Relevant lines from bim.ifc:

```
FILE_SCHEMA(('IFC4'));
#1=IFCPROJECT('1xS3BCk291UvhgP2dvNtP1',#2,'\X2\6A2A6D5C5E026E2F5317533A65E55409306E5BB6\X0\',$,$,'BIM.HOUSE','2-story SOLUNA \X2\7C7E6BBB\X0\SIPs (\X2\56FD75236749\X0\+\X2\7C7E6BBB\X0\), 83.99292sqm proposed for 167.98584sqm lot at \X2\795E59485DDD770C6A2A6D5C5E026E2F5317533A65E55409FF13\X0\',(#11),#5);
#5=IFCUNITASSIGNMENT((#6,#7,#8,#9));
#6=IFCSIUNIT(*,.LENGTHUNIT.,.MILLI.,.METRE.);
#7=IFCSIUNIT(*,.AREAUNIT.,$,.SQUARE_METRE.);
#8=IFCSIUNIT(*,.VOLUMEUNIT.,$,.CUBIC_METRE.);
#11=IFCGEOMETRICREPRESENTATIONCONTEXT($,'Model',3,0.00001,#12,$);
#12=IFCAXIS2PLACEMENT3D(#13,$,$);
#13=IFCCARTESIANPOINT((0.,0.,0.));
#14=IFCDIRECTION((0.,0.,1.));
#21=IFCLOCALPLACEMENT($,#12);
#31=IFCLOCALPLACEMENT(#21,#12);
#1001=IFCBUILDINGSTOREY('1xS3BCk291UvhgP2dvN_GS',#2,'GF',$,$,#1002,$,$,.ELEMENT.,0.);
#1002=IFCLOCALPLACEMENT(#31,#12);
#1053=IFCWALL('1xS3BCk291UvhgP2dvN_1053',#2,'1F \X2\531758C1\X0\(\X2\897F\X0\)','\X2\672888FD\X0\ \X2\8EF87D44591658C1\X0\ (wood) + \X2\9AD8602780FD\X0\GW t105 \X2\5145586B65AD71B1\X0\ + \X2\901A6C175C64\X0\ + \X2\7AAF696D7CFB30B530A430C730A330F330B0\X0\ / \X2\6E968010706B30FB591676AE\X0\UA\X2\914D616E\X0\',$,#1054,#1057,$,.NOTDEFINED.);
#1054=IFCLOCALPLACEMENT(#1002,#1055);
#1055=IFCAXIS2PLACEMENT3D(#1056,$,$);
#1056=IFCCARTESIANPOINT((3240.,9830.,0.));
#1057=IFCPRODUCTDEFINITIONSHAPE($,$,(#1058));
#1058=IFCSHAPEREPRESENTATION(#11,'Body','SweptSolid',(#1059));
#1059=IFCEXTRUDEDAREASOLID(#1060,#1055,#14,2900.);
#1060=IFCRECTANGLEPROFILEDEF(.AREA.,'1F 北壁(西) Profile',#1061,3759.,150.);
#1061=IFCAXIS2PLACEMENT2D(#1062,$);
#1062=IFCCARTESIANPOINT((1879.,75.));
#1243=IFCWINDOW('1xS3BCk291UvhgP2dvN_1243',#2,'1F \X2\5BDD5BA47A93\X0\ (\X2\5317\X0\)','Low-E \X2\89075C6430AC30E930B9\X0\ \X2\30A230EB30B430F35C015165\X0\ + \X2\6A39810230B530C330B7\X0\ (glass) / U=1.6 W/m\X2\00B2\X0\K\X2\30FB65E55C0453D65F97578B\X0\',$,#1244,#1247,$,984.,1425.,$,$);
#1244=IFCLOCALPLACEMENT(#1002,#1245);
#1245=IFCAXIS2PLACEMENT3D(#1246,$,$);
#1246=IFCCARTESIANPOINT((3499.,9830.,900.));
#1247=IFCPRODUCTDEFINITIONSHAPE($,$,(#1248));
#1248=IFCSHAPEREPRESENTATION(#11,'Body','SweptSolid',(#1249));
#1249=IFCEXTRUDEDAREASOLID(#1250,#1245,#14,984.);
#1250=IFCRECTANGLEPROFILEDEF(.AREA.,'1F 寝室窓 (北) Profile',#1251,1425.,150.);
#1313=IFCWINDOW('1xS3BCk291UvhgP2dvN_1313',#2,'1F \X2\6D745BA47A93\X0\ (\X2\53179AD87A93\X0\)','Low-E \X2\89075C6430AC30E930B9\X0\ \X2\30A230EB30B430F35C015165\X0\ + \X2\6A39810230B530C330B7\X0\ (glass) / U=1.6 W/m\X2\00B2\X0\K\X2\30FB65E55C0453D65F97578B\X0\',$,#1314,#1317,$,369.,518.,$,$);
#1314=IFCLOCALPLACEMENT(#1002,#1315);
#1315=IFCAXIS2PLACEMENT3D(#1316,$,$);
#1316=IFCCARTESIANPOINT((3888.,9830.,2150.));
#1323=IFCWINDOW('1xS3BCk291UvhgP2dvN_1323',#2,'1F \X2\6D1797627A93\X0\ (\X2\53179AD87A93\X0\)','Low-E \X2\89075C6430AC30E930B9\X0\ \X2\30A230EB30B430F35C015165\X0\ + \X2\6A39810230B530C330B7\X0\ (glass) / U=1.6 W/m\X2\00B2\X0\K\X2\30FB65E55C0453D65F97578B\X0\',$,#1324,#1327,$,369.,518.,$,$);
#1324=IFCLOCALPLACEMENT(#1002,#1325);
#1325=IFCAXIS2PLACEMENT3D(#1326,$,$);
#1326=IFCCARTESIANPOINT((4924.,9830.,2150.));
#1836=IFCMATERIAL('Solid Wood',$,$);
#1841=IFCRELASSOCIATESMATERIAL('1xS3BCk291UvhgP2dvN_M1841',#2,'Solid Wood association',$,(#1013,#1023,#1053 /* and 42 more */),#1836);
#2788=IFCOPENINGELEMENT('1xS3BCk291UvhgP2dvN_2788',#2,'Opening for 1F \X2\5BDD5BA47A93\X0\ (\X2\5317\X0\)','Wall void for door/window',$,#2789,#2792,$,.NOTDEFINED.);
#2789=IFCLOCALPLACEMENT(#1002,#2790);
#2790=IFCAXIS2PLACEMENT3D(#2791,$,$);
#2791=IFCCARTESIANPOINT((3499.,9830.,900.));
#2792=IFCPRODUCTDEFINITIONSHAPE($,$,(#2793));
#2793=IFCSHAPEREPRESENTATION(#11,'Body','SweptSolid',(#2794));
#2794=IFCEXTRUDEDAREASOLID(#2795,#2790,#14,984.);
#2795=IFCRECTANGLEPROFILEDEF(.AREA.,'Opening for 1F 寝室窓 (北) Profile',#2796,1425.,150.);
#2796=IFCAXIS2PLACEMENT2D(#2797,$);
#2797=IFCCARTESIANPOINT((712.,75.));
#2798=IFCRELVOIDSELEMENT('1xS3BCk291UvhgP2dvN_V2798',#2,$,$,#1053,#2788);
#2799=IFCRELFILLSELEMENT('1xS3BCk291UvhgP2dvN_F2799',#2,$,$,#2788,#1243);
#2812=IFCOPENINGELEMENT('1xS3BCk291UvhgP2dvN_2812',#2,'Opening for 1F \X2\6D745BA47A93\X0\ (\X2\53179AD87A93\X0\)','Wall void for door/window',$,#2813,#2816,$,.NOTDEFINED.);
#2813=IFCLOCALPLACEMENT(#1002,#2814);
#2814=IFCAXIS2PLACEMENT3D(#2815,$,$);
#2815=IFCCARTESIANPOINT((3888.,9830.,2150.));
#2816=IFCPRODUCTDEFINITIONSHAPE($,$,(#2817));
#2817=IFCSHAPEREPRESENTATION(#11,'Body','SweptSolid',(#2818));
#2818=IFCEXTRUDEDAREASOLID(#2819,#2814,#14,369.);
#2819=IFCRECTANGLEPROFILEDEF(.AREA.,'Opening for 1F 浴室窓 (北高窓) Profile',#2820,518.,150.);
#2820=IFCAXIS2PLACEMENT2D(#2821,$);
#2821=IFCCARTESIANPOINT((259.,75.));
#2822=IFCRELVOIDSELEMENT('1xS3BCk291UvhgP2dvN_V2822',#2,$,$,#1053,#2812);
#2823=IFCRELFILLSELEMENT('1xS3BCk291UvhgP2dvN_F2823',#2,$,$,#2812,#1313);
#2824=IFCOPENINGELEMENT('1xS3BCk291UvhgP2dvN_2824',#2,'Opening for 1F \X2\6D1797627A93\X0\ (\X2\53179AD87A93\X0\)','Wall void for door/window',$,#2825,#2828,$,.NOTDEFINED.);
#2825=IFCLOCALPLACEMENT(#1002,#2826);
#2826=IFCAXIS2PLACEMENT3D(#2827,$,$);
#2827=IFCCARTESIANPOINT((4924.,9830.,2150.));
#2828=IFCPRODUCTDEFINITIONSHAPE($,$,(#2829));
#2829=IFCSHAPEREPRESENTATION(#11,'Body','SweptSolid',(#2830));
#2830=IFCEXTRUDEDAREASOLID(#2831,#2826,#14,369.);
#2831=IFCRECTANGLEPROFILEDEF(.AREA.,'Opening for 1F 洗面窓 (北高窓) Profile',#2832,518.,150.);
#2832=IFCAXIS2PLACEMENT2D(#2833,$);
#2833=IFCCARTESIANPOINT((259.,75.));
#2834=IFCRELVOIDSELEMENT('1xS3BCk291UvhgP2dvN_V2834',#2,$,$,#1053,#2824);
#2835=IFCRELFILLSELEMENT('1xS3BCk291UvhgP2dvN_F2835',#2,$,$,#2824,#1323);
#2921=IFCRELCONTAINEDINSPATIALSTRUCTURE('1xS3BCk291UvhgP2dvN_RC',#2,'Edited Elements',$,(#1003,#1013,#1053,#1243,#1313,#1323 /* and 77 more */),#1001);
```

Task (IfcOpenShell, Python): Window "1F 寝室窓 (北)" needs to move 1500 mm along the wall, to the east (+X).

```python
import ifcopenshell
import ifcopenshell.api.geometry
import ifcopenshell.util.placement
import ifcopenshell.util.unit

model = ifcopenshell.open("bim.ifc")
unit_scale = ifcopenshell.util.unit.calculate_unit_scale(model)

window = model.by_id(1243)
opening = window.FillsVoids[0].RelatingOpeningElement
wall = opening.VoidsElements[0].RelatingBuildingElement

wall_matrix = ifcopenshell.util.placement.get_local_placement(wall.ObjectPlacement)
shift = wall_matrix[:3, 0] * 1.5 / unit_scale
before = ifcopenshell.util.placement.get_local_placement(window.ObjectPlacement)[:3, 3].copy()

# The window is not placed relative to its opening, so move both.
for product in (opening, window):
    matrix = ifcopenshell.util.placement.get_local_placement(product.ObjectPlacement)
    matrix[:3, 3] += shift
    ifcopenshell.api.geometry.edit_object_placement(model, product=product, matrix=matrix, is_si=False)

after = ifcopenshell.util.placement.get_local_placement(window.ObjectPlacement)[:3, 3]
print("window moved by", (after - before).round(3) + 0.0)

model.write("bim-out.ifc")
```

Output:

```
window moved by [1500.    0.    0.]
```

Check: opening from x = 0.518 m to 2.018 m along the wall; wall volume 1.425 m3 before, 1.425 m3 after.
